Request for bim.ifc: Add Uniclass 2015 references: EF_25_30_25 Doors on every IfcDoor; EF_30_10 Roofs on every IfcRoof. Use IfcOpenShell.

First a look at what the model holds.

```python
import ifcopenshell

model = ifcopenshell.open("bim.ifc")
print(model.schema)
print("classifications:", [c.Name for c in model.by_type("IfcClassification")])
for ifc_class in ("IfcDoor", "IfcRoof", "IfcStair", "IfcWall", "IfcWindow"):
    print(ifc_class, len(model.by_type(ifc_class)))
```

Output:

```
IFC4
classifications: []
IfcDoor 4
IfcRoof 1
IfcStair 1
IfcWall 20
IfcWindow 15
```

```python
import ifcopenshell
import ifcopenshell.api.classification

model = ifcopenshell.open("bim.ifc")

system = ifcopenshell.api.classification.add_classification(model, classification="Uniclass 2015")

codes = {
    "IfcDoor": ("EF_25_30_25", "Doors"),
    "IfcRoof": ("EF_30_10", "Roofs"),
}
for ifc_class, (code, name) in codes.items():
    products = model.by_type(ifc_class)
    ifcopenshell.api.classification.add_reference(
        model, products=products, classification=system, identification=code, name=name
    )
    print(code, len(products))

model.write("bim-out.ifc")
```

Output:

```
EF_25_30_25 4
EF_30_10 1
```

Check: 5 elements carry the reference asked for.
